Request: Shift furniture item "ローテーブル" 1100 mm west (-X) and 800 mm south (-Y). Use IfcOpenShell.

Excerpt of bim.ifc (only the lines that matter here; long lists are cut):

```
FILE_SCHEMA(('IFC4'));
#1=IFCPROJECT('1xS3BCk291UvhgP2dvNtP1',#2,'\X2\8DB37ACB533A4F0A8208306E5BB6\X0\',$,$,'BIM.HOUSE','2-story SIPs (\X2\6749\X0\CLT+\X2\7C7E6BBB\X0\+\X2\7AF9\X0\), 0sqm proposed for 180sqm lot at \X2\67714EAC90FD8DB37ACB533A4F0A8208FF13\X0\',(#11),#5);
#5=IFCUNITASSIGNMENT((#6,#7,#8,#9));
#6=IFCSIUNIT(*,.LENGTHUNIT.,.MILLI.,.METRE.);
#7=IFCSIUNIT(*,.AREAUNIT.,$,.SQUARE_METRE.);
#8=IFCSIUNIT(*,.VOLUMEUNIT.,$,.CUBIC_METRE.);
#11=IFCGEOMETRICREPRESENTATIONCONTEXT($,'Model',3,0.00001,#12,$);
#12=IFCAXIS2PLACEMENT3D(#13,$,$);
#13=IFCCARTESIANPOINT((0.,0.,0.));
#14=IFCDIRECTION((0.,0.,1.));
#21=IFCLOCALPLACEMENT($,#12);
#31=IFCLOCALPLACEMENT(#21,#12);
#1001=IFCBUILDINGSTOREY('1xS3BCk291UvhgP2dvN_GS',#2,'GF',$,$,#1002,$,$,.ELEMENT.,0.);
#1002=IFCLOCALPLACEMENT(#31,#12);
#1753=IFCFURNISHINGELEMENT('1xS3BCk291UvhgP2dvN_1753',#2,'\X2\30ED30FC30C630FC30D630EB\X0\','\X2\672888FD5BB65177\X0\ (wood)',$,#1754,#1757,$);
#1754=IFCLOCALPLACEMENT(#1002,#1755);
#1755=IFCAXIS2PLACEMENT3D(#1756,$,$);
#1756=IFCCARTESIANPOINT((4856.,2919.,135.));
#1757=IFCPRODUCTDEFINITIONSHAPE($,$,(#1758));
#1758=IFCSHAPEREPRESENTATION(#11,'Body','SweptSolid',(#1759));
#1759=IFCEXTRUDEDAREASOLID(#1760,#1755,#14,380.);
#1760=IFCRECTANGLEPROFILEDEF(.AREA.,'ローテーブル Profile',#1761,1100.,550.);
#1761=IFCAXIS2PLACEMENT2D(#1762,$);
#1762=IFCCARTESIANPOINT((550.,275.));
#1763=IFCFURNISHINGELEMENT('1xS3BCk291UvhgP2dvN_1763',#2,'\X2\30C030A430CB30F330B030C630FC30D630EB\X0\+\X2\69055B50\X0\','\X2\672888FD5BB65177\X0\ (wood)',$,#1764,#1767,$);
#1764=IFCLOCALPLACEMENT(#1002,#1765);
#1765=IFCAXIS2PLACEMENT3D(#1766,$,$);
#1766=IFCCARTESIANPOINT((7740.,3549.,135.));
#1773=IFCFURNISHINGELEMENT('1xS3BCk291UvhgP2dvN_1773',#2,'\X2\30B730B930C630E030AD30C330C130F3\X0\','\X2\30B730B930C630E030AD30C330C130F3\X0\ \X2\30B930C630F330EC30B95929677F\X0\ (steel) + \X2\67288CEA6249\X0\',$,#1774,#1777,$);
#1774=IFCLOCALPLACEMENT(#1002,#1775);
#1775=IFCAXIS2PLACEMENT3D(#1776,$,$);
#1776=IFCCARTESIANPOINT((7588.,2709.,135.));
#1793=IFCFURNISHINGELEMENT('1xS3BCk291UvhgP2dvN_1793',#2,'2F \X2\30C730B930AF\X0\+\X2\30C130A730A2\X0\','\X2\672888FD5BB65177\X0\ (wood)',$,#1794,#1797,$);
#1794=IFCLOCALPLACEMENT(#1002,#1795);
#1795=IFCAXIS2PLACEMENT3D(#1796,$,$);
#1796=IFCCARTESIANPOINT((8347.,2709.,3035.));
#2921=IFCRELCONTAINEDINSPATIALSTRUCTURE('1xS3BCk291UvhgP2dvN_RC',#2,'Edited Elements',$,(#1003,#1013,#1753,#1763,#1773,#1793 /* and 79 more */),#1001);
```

```python
import ifcopenshell
import ifcopenshell.api.geometry
import ifcopenshell.util.placement
import ifcopenshell.util.unit

model = ifcopenshell.open("bim.ifc")
unit_scale = ifcopenshell.util.unit.calculate_unit_scale(model)

item = model.by_id(1753)
matrix = ifcopenshell.util.placement.get_local_placement(item.ObjectPlacement)
matrix[0, 3] -= 1.1 / unit_scale
matrix[1, 3] -= 0.8 / unit_scale
ifcopenshell.api.geometry.edit_object_placement(model, product=item, matrix=matrix, is_si=False)

print(ifcopenshell.util.placement.get_local_placement(item.ObjectPlacement).round(3) + 0.0)

model.write("bim_v2.ifc")
```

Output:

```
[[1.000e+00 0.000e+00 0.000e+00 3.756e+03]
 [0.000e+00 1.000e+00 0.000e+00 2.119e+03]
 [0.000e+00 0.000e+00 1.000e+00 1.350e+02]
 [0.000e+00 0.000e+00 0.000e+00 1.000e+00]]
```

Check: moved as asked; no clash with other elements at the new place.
